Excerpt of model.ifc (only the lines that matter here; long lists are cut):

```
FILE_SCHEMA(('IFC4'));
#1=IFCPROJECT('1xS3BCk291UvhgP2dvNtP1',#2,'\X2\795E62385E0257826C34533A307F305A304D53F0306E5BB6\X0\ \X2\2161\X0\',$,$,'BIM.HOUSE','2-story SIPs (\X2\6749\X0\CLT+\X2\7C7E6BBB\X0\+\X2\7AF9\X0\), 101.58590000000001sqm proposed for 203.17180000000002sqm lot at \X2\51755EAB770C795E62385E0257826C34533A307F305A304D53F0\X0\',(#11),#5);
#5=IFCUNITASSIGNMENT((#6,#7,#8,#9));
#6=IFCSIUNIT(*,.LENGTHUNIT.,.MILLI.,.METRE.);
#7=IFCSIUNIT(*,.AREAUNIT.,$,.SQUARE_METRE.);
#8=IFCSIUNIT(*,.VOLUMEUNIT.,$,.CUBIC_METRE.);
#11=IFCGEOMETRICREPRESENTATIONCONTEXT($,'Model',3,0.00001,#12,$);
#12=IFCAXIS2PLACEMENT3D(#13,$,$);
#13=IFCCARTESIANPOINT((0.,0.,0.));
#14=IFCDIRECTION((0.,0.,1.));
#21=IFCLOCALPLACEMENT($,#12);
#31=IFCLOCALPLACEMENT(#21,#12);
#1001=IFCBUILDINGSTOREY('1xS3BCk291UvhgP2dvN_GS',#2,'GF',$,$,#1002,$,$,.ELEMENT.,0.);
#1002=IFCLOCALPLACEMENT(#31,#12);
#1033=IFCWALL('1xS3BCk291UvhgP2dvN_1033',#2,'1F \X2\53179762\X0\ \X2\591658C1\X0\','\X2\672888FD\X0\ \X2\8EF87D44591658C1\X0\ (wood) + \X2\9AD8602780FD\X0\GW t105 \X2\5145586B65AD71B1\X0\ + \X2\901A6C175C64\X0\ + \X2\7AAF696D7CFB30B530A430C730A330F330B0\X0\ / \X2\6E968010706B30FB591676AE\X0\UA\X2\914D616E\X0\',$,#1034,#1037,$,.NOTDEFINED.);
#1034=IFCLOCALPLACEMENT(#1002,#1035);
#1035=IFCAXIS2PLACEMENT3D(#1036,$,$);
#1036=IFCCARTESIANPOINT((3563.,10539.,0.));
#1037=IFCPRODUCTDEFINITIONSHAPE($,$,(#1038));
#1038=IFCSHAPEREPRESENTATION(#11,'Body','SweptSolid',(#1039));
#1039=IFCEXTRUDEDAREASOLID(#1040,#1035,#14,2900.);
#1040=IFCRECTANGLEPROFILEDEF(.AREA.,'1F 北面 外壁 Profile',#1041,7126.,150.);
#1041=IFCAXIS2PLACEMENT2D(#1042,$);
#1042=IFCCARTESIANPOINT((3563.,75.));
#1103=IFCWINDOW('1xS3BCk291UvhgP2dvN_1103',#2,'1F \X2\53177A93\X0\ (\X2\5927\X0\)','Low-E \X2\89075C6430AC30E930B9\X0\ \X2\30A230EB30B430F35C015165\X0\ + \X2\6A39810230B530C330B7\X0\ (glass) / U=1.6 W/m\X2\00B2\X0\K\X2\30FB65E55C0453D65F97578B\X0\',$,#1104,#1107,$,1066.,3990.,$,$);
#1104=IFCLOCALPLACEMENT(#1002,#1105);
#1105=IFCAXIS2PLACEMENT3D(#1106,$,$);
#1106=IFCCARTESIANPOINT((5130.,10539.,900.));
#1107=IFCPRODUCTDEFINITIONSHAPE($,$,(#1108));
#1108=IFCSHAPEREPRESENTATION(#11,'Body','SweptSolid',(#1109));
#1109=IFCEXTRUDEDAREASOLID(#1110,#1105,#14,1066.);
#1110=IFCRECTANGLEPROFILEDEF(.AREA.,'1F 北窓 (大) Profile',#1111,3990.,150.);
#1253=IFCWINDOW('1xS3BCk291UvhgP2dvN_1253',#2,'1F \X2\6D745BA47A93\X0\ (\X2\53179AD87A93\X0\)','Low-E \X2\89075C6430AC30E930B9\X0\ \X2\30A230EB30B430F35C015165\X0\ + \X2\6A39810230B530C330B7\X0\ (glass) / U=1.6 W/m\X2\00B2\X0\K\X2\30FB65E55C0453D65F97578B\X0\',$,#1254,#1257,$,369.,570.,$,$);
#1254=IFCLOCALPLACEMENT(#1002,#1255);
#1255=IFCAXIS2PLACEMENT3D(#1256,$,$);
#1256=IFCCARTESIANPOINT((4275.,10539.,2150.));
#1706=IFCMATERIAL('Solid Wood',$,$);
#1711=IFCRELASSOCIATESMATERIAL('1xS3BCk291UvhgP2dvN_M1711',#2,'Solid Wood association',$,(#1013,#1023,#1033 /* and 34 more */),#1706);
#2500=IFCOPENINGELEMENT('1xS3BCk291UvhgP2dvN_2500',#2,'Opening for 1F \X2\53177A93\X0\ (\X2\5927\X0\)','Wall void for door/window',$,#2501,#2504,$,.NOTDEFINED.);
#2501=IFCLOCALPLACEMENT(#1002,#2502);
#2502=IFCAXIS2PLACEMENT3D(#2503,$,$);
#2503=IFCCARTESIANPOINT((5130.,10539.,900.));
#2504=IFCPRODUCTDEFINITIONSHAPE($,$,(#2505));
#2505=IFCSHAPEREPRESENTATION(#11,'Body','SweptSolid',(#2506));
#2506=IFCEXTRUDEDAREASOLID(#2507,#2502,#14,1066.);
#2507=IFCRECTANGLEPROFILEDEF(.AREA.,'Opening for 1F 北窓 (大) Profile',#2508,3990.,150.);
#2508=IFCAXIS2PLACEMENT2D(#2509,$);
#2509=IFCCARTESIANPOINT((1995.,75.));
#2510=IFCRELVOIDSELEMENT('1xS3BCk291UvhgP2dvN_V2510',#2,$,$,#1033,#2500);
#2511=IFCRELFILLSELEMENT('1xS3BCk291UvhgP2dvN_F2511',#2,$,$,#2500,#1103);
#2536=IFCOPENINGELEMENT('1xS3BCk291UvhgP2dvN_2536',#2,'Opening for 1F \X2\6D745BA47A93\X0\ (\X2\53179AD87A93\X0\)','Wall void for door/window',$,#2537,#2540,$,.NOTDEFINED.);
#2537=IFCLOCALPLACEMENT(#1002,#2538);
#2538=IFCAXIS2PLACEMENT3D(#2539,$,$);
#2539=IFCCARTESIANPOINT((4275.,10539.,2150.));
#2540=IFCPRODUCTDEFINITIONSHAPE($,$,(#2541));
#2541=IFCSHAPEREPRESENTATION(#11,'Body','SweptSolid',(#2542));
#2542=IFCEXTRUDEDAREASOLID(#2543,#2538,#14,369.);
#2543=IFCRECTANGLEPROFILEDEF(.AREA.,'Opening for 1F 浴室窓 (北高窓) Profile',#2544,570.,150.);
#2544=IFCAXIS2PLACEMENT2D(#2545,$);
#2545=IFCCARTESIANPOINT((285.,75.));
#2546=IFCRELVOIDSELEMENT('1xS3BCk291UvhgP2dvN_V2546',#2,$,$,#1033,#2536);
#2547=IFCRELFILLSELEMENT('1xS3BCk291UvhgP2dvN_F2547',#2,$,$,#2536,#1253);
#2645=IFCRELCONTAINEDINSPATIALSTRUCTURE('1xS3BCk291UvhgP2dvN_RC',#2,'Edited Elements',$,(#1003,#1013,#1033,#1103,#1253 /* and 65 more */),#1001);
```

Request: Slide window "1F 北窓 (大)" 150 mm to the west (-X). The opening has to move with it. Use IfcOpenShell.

```python
import ifcopenshell
import ifcopenshell.api.geometry
import ifcopenshell.util.placement
import ifcopenshell.util.unit

model = ifcopenshell.open("model.ifc")
unit_scale = ifcopenshell.util.unit.calculate_unit_scale(model)

window = model.by_guid("1xS3BCk291UvhgP2dvN_1103")
opening = window.FillsVoids[0].RelatingOpeningElement
wall = opening.VoidsElements[0].RelatingBuildingElement

wall_matrix = ifcopenshell.util.placement.get_local_placement(wall.ObjectPlacement)
shift = wall_matrix[:3, 0] * -0.15 / unit_scale
before = ifcopenshell.util.placement.get_local_placement(window.ObjectPlacement)[:3, 3].copy()

# The window is not placed relative to its opening, so move both.
for product in (opening, window):
    matrix = ifcopenshell.util.placement.get_local_placement(product.ObjectPlacement)
    matrix[:3, 3] += shift
    ifcopenshell.api.geometry.edit_object_placement(model, product=product, matrix=matrix, is_si=False)

after = ifcopenshell.util.placement.get_local_placement(window.ObjectPlacement)[:3, 3]
print("window moved by", (after - before).round(3) + 0.0)

model.write("model_updated.ifc")
```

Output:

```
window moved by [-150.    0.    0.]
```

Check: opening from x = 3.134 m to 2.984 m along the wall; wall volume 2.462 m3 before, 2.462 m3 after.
